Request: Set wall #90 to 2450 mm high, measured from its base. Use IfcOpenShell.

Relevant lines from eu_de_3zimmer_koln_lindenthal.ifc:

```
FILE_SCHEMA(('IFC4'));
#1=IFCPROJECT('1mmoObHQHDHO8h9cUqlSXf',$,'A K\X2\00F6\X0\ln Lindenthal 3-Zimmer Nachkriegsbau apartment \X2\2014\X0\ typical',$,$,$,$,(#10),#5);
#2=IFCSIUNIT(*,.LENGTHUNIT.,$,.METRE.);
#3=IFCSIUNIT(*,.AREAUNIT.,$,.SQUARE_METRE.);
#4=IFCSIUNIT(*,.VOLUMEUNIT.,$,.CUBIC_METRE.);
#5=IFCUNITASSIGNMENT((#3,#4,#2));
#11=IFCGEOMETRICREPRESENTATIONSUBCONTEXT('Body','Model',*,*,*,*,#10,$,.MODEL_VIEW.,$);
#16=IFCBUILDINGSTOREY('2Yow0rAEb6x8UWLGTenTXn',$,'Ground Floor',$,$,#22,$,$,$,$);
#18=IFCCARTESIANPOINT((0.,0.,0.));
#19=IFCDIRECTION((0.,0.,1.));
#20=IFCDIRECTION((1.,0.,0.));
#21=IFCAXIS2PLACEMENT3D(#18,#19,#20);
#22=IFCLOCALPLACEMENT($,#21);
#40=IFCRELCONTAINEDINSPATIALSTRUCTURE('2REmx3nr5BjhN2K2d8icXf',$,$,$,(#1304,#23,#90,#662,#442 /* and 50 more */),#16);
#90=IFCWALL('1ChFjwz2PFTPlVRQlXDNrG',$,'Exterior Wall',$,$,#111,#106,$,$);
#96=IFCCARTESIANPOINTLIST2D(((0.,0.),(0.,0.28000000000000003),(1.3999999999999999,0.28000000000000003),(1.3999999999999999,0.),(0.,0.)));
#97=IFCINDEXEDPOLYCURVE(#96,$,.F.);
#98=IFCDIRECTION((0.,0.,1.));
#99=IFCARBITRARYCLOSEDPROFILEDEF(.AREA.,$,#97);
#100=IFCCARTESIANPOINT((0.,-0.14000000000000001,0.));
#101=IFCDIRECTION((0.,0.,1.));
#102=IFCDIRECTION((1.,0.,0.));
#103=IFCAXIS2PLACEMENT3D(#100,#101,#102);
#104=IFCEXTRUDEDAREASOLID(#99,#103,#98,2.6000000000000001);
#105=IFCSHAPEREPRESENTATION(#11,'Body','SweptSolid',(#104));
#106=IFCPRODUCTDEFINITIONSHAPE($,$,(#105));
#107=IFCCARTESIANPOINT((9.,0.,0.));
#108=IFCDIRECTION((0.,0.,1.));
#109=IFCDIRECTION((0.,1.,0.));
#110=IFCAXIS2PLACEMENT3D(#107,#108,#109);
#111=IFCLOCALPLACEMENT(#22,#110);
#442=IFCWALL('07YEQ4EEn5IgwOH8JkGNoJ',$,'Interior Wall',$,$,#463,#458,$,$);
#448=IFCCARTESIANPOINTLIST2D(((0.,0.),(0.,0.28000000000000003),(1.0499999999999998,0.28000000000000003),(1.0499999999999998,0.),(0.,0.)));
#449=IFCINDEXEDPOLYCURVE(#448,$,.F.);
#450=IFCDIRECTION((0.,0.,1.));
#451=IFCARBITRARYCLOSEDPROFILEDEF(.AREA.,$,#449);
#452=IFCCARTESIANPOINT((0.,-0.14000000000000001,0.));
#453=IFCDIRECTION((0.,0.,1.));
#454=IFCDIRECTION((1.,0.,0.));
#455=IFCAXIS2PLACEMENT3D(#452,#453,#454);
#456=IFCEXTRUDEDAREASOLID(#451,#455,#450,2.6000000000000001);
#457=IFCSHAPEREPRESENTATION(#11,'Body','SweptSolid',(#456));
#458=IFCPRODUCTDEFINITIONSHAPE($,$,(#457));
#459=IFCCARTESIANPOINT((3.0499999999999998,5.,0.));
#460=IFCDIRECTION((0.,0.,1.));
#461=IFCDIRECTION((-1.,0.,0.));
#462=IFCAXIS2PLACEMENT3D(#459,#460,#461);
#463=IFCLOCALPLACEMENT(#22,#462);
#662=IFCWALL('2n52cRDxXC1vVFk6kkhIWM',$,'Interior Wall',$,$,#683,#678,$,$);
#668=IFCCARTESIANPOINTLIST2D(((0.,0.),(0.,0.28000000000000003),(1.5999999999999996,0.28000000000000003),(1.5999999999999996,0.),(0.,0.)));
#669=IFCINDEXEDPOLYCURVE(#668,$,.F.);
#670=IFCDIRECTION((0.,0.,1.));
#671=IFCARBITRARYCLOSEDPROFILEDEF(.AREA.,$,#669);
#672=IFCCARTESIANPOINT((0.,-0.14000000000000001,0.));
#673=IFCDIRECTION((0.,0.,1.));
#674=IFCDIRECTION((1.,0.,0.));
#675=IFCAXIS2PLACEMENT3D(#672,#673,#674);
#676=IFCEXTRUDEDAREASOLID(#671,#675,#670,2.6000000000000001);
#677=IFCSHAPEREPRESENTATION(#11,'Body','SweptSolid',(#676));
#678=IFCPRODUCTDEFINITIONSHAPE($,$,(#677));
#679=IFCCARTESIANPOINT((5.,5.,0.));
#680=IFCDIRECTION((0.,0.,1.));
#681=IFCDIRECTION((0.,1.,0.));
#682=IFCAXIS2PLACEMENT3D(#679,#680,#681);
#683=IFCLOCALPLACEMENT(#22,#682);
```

```python
import ifcopenshell
import ifcopenshell.geom
import ifcopenshell.util.representation
import ifcopenshell.util.shape

model = ifcopenshell.open("eu_de_3zimmer_koln_lindenthal.ifc")
settings = ifcopenshell.geom.settings()


def volume(element):
    """Net volume in cubic metres, openings subtracted."""
    shape = ifcopenshell.geom.create_shape(settings, element)
    return ifcopenshell.util.shape.get_volume(shape.geometry)


wall = model.by_guid("1ChFjwz2PFTPlVRQlXDNrG")
before = volume(wall)

body = ifcopenshell.util.representation.get_representation(wall, "Model", "Body")
solid = body.Items[0]
old_height = solid.Depth
solid.Depth = 2.45
after = volume(wall)

print(f"height {old_height:g} -> {solid.Depth:g}, volume {before:.3f} -> {after:.3f} m3")

model.write("eu_de_3zimmer_koln_lindenthal_v2.ifc")
```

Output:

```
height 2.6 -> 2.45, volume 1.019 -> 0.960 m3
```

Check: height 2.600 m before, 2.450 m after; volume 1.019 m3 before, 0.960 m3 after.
